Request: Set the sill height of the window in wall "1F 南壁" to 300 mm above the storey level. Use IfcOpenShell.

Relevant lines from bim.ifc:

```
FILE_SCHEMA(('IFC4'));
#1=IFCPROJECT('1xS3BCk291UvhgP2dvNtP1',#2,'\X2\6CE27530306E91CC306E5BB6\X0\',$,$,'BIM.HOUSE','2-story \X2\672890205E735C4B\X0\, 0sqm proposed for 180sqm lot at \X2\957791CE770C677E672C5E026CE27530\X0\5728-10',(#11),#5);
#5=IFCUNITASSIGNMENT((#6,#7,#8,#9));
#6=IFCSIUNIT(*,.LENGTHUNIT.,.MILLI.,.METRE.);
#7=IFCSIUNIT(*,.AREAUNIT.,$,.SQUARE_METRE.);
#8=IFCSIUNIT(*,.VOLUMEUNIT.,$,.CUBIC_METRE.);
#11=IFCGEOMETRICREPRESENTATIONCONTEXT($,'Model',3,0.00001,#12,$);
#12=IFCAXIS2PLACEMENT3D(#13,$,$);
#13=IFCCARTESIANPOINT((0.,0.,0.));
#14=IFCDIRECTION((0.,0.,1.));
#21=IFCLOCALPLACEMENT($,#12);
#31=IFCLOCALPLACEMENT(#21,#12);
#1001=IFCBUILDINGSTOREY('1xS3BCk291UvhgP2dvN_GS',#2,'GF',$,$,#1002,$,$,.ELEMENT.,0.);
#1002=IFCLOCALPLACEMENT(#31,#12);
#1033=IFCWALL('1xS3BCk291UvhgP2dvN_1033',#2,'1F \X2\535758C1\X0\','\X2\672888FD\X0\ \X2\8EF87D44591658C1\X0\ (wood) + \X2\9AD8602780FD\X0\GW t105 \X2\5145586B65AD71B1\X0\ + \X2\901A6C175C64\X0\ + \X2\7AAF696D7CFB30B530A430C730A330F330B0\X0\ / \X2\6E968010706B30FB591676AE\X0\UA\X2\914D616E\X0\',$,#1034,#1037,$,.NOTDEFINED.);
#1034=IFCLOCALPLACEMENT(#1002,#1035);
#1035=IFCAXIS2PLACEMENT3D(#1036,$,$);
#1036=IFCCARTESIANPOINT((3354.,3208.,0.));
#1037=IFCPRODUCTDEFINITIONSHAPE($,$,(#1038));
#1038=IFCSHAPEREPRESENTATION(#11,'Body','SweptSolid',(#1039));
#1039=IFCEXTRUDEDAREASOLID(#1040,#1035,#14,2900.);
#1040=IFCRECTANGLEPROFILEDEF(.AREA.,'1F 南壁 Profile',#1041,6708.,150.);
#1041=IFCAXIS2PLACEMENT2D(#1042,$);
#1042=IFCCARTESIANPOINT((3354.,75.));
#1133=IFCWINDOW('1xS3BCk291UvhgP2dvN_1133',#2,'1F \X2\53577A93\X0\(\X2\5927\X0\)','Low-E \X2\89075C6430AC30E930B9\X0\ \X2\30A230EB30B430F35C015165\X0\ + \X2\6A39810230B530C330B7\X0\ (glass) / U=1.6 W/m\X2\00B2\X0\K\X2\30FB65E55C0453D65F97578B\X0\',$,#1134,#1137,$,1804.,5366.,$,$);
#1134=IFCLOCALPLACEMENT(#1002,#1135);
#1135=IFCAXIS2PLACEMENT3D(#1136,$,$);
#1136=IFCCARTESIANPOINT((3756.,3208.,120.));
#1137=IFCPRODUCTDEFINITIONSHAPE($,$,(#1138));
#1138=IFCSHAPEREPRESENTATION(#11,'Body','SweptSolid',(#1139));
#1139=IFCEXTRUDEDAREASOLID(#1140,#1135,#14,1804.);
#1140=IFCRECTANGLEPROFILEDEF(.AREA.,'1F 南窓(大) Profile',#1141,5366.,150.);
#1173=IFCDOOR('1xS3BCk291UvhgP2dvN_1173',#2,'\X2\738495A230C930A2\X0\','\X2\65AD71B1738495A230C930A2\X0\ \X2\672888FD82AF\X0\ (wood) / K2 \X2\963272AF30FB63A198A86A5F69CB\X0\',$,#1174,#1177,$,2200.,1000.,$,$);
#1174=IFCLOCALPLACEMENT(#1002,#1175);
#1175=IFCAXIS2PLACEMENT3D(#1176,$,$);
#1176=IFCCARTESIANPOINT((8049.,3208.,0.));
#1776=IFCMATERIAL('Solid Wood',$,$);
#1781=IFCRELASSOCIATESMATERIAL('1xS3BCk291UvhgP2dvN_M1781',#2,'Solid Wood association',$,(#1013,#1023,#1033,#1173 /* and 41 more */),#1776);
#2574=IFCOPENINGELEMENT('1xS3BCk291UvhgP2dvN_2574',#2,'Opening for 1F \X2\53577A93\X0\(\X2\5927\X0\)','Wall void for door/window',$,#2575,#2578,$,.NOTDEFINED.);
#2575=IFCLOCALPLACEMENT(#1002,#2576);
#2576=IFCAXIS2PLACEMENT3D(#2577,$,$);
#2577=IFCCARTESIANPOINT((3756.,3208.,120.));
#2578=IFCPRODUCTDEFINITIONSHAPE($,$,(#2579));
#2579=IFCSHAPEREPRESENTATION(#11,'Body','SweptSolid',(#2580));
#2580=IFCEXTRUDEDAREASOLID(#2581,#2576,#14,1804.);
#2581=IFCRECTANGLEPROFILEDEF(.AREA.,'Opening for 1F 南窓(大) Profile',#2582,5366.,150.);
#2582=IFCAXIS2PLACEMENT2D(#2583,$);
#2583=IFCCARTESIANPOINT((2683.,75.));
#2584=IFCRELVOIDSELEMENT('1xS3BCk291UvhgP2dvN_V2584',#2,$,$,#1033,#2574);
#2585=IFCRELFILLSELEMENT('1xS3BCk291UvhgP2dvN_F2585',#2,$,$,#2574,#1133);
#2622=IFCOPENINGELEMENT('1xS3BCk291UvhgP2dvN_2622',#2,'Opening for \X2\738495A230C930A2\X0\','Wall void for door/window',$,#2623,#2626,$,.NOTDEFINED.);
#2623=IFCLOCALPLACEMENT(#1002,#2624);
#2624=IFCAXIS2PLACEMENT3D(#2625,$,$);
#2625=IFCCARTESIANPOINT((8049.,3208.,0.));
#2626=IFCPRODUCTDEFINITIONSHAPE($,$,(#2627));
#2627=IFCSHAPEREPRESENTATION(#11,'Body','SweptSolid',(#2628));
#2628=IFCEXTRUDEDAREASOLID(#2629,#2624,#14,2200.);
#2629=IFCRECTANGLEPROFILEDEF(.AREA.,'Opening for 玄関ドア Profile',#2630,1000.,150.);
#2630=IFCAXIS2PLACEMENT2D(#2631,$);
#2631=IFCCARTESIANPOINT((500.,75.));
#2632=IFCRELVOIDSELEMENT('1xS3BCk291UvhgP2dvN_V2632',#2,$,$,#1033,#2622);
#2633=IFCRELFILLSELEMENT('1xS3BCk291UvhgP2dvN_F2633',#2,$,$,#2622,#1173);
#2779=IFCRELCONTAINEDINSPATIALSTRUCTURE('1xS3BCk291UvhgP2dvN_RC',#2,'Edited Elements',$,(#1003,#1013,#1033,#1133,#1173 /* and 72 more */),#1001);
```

```python
import numpy as np
import ifcopenshell
import ifcopenshell.api.geometry
import ifcopenshell.geom
import ifcopenshell.util.element
import ifcopenshell.util.placement
import ifcopenshell.util.shape
import ifcopenshell.util.unit

model = ifcopenshell.open("bim.ifc")
unit_scale = ifcopenshell.util.unit.calculate_unit_scale(model)

window = model.by_guid("1xS3BCk291UvhgP2dvN_1133")
opening = window.FillsVoids[0].RelatingOpeningElement
storey = ifcopenshell.util.element.get_container(window, ifc_class="IfcBuildingStorey")
level = ifcopenshell.util.placement.get_local_placement(storey.ObjectPlacement)[2, 3]

# The opening's origin need not be at the sill, so measure its lowest point.
shape = ifcopenshell.geom.create_shape(ifcopenshell.geom.settings(), opening)
bottom = ifcopenshell.util.shape.get_shape_bottom_elevation(shape, shape.geometry) / unit_scale
dz = level + 300.0 - bottom

shift = np.array([0.0, 0.0, dz])
# The window is not placed relative to its opening, so move both.
for product in (opening, window):
    matrix = ifcopenshell.util.placement.get_local_placement(product.ObjectPlacement)
    matrix[:3, 3] += shift
    ifcopenshell.api.geometry.edit_object_placement(model, product=product, matrix=matrix, is_si=False)

print(f"moved by {dz * unit_scale:+.3f} m")

model.write("bim_updated.ifc")
```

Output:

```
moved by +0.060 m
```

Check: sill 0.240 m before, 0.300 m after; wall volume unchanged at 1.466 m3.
